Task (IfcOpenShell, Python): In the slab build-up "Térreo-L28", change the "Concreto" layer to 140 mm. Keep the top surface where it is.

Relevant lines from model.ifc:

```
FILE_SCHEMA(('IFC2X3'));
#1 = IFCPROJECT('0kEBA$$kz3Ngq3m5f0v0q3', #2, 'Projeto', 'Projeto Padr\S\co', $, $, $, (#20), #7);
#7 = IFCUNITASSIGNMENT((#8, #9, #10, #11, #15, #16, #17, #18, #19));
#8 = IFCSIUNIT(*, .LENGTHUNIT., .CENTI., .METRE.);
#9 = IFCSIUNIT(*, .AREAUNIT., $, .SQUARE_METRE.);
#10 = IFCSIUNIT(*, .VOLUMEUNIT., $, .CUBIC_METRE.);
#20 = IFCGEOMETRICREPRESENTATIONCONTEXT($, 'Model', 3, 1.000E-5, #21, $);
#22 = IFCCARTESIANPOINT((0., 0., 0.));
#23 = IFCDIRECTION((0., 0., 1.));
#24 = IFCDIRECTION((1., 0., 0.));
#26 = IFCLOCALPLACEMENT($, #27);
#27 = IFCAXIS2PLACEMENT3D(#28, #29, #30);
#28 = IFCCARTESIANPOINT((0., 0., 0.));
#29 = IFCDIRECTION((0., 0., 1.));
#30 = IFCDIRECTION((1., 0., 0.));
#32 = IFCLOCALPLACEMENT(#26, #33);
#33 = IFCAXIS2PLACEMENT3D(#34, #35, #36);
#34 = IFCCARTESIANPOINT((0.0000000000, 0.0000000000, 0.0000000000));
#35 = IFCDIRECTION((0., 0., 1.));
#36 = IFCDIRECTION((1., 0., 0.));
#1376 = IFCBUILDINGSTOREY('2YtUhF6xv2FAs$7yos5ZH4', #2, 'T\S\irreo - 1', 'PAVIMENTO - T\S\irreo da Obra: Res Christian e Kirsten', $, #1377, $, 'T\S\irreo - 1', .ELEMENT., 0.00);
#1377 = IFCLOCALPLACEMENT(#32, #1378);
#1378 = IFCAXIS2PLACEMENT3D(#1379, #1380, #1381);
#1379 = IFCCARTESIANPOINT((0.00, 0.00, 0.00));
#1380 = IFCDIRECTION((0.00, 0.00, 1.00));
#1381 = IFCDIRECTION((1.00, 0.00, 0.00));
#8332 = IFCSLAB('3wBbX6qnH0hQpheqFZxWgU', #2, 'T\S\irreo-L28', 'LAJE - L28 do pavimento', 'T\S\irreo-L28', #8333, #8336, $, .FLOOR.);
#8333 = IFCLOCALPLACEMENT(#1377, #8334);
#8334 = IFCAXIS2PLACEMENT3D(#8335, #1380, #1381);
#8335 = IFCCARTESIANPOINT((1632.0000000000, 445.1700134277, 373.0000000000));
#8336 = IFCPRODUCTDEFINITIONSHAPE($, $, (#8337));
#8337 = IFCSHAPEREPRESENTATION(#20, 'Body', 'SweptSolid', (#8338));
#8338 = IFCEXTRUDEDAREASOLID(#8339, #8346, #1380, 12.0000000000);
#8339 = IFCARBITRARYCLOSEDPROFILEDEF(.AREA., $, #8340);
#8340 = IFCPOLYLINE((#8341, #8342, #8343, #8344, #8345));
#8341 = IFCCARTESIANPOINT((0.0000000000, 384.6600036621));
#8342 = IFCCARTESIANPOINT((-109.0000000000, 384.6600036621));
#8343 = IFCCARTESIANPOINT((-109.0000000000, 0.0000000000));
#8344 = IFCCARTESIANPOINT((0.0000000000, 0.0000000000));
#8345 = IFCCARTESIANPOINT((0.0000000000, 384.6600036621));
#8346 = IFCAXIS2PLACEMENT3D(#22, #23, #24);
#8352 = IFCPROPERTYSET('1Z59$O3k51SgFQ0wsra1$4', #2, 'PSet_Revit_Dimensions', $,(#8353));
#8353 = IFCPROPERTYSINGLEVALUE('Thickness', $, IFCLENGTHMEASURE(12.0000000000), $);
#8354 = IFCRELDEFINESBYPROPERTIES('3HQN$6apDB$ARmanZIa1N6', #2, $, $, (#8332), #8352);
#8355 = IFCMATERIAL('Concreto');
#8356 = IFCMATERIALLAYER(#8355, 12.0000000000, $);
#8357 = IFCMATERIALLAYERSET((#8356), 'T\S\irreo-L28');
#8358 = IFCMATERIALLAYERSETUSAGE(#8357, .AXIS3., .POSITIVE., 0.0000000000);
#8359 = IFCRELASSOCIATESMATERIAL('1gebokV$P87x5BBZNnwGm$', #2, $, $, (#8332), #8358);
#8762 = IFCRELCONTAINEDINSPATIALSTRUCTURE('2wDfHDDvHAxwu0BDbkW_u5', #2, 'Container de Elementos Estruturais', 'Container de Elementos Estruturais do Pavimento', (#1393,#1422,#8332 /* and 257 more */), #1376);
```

```python
import ifcopenshell
import ifcopenshell.api.pset
import ifcopenshell.util.element
import ifcopenshell.util.unit

model = ifcopenshell.open("model.ifc")
unit_scale = ifcopenshell.util.unit.calculate_unit_scale(model)

layer_set = model.by_id(8357)
layer = next(l for l in layer_set.MaterialLayers if l.Material and l.Material.Name == "Concreto")
change = 0.14 / unit_scale - layer.LayerThickness
layer.LayerThickness += change

# Geometry does not follow the layer set by itself.
slabs = [e for e in ifcopenshell.util.element.get_elements_by_material(model, layer_set) if e.is_a("IfcSlab")]
for slab in sorted(slabs, key=lambda e: e.id()):
    body = next(r for r in slab.Representation.Representations if r.RepresentationIdentifier == "Body")
    solid = body.Items[0]
    old_depth = solid.Depth
    solid.Depth += change
    # Extruded upwards: lower the start of the extrusion so the top stays.
    x, y, z = solid.Position.Location.Coordinates
    solid.Position.Location = model.createIfcCartesianPoint((x, y, z - change))
    pset = model.by_id(ifcopenshell.util.element.get_pset(slab, "PSet_Revit_Dimensions", should_inherit=False)["id"])
    ifcopenshell.api.pset.edit_pset(model, pset=pset, properties={
        "Thickness": model.create_entity("IfcLengthMeasure", solid.Depth),
    })
    print(slab.id(), f"{old_depth:g} -> {solid.Depth:g}")

# The layers are counted up from the underside, which has moved.
for usage in {ifcopenshell.util.element.get_material(slab) for slab in slabs}:
    usage.OffsetFromReferenceLine -= change

model.write("model-out.ifc")
```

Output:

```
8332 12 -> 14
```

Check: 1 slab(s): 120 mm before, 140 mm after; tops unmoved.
